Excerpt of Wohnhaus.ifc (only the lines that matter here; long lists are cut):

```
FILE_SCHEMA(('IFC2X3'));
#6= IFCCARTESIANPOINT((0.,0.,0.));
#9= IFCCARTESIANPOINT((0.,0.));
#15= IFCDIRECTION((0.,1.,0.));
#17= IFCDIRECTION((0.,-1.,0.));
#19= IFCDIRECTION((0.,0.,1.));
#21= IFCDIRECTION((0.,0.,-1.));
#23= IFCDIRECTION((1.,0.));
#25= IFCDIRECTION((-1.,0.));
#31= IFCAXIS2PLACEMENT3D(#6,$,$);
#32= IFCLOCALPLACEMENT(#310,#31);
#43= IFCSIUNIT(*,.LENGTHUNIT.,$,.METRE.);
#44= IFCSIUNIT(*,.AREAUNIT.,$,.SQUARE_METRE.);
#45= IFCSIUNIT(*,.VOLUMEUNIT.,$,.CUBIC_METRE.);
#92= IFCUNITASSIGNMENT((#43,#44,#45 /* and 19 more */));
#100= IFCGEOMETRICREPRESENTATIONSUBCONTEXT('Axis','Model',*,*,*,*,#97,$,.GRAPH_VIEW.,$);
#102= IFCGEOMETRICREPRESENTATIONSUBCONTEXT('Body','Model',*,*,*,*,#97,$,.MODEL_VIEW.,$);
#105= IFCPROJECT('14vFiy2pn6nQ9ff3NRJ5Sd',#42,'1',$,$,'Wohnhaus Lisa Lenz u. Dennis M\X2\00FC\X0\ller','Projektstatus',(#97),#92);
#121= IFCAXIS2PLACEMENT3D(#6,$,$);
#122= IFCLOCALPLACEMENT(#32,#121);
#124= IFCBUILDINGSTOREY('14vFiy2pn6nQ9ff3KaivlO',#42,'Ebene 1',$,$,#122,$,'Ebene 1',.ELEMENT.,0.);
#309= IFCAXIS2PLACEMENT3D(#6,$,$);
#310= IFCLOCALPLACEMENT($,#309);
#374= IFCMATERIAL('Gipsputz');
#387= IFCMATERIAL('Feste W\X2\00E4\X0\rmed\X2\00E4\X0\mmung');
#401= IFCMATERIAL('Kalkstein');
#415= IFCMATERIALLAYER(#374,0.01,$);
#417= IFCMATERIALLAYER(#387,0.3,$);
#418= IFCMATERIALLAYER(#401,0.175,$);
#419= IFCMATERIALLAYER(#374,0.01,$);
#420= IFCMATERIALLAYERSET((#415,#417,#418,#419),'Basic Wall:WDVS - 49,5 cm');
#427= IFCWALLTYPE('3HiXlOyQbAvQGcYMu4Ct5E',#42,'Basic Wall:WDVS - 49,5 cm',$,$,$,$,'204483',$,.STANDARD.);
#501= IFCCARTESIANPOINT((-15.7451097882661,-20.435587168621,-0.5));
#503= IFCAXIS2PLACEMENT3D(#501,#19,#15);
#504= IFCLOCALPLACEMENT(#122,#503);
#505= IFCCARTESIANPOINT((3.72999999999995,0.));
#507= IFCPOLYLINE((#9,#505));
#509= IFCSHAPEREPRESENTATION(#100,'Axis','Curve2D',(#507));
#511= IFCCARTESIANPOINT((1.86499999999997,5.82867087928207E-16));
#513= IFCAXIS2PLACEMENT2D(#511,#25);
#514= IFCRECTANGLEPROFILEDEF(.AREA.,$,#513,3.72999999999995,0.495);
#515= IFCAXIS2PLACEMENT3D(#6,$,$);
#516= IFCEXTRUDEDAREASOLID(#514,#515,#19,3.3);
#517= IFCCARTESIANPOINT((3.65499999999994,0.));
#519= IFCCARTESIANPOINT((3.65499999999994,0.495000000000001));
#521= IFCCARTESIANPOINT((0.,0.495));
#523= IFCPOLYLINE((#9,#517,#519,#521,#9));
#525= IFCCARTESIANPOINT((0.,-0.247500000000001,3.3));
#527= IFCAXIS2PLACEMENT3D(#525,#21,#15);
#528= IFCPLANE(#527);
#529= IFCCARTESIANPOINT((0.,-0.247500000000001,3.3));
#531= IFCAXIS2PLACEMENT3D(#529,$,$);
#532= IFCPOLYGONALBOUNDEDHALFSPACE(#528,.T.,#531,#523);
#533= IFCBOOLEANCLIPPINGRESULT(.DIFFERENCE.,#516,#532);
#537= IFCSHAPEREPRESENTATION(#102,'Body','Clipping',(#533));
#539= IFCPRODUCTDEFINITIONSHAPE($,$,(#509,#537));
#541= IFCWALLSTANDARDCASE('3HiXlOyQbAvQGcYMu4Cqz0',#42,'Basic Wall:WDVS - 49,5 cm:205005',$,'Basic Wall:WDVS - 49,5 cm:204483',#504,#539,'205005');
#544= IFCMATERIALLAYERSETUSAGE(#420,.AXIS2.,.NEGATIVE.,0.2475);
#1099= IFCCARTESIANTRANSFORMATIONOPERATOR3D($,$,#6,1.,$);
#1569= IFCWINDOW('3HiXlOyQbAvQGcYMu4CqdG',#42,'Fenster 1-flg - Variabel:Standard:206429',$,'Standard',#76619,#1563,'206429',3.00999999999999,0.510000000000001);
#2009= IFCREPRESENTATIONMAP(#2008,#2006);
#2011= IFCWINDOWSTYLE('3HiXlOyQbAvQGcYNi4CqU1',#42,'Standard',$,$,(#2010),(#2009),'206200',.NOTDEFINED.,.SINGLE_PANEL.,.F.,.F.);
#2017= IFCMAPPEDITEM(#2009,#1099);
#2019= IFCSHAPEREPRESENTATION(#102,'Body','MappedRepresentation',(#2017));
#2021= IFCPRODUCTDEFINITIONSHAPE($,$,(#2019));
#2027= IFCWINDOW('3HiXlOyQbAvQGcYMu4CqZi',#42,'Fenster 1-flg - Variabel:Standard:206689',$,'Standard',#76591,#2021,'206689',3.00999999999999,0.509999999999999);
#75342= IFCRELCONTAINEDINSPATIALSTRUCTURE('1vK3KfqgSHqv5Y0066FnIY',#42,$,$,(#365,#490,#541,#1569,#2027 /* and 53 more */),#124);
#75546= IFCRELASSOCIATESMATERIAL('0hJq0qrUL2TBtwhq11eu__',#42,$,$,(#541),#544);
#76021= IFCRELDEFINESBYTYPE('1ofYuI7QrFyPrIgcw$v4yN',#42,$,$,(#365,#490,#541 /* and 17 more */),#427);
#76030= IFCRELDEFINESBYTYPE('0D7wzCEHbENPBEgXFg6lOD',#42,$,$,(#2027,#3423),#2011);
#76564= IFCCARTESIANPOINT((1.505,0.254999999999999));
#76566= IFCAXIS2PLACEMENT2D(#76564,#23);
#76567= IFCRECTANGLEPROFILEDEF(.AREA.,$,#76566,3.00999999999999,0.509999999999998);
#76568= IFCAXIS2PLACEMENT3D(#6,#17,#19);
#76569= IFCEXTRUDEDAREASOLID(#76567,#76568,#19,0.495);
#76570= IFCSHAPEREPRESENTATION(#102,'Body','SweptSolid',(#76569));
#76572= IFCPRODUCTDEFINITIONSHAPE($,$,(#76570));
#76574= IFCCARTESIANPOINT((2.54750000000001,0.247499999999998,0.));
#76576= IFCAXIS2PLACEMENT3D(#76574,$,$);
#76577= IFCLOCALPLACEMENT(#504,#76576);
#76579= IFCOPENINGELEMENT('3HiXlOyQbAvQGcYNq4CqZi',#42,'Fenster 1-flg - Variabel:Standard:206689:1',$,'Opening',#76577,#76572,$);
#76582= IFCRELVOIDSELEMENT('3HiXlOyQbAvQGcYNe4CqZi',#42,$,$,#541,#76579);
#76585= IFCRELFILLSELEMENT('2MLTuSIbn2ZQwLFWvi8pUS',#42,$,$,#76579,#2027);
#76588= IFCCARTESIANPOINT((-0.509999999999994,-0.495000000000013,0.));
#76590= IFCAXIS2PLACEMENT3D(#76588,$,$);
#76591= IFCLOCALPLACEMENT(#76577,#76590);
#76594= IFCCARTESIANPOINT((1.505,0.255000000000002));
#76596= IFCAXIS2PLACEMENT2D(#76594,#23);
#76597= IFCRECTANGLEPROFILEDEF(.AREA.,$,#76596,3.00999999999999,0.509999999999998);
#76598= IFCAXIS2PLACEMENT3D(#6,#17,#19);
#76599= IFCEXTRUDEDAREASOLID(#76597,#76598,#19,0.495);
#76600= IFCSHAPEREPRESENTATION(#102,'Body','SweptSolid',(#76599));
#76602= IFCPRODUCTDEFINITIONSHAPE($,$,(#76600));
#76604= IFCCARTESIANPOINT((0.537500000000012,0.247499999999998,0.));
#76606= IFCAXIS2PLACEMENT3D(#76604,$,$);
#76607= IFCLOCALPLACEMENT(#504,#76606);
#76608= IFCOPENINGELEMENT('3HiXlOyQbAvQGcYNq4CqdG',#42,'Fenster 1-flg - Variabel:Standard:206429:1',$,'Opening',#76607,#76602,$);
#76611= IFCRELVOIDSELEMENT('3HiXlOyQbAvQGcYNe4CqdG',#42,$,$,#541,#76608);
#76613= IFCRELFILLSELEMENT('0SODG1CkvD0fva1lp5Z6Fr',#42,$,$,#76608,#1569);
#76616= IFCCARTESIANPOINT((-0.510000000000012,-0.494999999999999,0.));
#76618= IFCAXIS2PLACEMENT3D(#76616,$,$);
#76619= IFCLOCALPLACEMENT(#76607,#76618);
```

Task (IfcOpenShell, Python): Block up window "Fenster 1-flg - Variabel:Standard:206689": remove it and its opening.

```python
import ifcopenshell
import ifcopenshell.api.feature
import ifcopenshell.api.root
import ifcopenshell.geom
import ifcopenshell.util.shape

model = ifcopenshell.open("Wohnhaus.ifc")
settings = ifcopenshell.geom.settings()


def volume(element):
    """Net volume in cubic metres, openings subtracted."""
    shape = ifcopenshell.geom.create_shape(settings, element)
    return ifcopenshell.util.shape.get_volume(shape.geometry)


window = model.by_guid("3HiXlOyQbAvQGcYMu4CqZi")
opening = window.FillsVoids[0].RelatingOpeningElement
wall = opening.VoidsElements[0].RelatingBuildingElement
before = volume(wall)

ifcopenshell.api.root.remove_product(model, product=window)
ifcopenshell.api.feature.remove_feature(model, feature=opening)

after = volume(wall)

print(f"wall volume {before:.3f} -> {after:.3f} m3")

model.write("Wohnhaus_rev.ifc")
```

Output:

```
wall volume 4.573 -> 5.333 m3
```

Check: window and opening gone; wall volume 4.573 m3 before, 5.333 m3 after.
